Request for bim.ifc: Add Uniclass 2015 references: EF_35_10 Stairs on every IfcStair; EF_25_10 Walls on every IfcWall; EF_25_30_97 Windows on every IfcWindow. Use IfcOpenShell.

First a look at what the model holds.

```python
import ifcopenshell

model = ifcopenshell.open("bim.ifc")
print(model.schema)
print("classifications:", [c.Name for c in model.by_type("IfcClassification")])
for ifc_class in ("IfcDoor", "IfcRoof", "IfcStair", "IfcWall", "IfcWindow"):
    print(ifc_class, len(model.by_type(ifc_class)))
```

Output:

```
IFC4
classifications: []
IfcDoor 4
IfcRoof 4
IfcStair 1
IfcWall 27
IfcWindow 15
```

```python
import ifcopenshell
import ifcopenshell.api.classification

model = ifcopenshell.open("bim.ifc")

system = ifcopenshell.api.classification.add_classification(model, classification="Uniclass 2015")

codes = {
    "IfcStair": ("EF_35_10", "Stairs"),
    "IfcWall": ("EF_25_10", "Walls"),
    "IfcWindow": ("EF_25_30_97", "Windows"),
}
for ifc_class, (code, name) in codes.items():
    products = model.by_type(ifc_class)
    ifcopenshell.api.classification.add_reference(
        model, products=products, classification=system, identification=code, name=name
    )
    print(code, len(products))

model.write("bim_edited.ifc")
```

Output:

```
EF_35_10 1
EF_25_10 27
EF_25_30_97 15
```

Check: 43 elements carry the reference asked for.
